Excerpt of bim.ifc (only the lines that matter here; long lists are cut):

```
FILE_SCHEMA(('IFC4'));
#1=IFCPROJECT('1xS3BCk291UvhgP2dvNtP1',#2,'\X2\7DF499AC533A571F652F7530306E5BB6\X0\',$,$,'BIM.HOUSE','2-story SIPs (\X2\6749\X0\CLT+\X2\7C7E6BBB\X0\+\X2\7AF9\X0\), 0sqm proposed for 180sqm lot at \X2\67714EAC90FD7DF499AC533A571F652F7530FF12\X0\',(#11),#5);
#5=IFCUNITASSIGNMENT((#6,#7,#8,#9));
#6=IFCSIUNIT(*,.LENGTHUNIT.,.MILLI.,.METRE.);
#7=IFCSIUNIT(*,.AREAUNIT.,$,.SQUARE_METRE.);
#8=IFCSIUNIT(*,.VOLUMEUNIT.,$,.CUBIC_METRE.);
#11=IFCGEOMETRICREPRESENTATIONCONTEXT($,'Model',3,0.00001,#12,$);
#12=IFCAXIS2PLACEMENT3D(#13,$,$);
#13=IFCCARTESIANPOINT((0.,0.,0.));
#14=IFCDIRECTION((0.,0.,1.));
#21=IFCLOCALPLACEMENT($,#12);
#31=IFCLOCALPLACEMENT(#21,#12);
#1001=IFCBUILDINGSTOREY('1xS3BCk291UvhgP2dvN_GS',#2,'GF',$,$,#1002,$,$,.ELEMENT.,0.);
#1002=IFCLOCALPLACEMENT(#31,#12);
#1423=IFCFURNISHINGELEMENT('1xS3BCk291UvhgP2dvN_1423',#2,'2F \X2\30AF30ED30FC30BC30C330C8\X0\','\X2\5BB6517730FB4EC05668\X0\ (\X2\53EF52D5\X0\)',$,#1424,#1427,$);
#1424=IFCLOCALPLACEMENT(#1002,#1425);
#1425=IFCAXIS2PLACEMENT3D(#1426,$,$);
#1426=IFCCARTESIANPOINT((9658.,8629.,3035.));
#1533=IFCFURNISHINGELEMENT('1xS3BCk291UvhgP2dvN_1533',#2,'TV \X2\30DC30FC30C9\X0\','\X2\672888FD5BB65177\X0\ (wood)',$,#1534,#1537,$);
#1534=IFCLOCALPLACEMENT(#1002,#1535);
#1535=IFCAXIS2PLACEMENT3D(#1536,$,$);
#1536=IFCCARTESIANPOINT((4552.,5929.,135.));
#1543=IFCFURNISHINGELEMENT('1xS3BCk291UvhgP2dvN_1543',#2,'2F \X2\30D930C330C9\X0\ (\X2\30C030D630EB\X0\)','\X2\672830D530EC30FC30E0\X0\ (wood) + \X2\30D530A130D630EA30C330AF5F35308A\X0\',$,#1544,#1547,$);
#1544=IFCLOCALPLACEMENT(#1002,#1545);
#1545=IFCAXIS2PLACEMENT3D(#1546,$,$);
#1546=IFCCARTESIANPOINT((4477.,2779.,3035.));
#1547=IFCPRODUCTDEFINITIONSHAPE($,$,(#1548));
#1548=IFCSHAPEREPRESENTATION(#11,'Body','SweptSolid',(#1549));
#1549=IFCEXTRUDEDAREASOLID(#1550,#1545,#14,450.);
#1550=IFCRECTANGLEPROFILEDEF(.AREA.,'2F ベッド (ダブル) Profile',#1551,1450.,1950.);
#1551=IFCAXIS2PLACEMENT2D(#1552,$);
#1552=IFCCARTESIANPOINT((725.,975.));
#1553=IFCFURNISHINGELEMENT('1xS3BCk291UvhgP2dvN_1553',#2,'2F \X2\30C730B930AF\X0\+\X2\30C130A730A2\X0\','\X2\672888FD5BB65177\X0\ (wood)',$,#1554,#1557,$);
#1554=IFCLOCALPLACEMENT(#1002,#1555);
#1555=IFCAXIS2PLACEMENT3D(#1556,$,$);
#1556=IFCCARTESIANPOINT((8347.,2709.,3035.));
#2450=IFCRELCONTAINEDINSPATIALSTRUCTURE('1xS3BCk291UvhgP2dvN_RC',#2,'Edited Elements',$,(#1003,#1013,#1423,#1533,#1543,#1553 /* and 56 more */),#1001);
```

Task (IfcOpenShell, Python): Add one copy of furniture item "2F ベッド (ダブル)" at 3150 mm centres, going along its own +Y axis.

```python
import ifcopenshell
import ifcopenshell.api.geometry
import ifcopenshell.api.root
import ifcopenshell.util.element
import ifcopenshell.util.placement
import ifcopenshell.util.unit

model = ifcopenshell.open("bim.ifc")
unit_scale = ifcopenshell.util.unit.calculate_unit_scale(model)


def reuse_history(source, copy):
    """copy_class also copies each property set's owner history, people and application; keep the originals."""
    for rel in copy.IsDefinedBy:
        if rel.is_a("IfcRelDefinesByProperties") and (history := rel.RelatingPropertyDefinition.OwnerHistory):
            rel.RelatingPropertyDefinition.OwnerHistory = source.OwnerHistory
            ifcopenshell.util.element.remove_deep2(model, history)


source = model.by_guid("1xS3BCk291UvhgP2dvN_1543")
base = ifcopenshell.util.placement.get_local_placement(source.ObjectPlacement)
step = base[:3, 1] * 3.15 / unit_scale

for i in range(1, 2):
    copy = ifcopenshell.api.root.copy_class(model, product=source)
    copy.Representation = ifcopenshell.util.element.copy_deep(
        model, source.Representation, exclude=["IfcGeometricRepresentationContext", "IfcRepresentationMap"]
    )
    reuse_history(source, copy)
    matrix = base.copy()
    matrix[:3, 3] += i * step
    print("added at", matrix[:3, 3].round(3) + 0.0)
    ifcopenshell.api.geometry.edit_object_placement(model, product=copy, matrix=matrix, is_si=False)

model.write("bim_rev.ifc")
```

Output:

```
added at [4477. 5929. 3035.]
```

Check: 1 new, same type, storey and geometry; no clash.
